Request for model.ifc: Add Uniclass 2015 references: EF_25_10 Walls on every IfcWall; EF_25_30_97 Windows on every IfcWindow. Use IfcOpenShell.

First a look at what the model holds.

```python
import ifcopenshell

model = ifcopenshell.open("model.ifc")
print(model.schema)
print("classifications:", [c.Name for c in model.by_type("IfcClassification")])
for ifc_class in ("IfcDoor", "IfcRoof", "IfcStair", "IfcWall", "IfcWindow"):
    print(ifc_class, len(model.by_type(ifc_class)))
```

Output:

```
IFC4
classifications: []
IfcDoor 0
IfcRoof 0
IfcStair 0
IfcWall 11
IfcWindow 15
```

```python
import ifcopenshell
import ifcopenshell.api.classification

model = ifcopenshell.open("model.ifc")

system = ifcopenshell.api.classification.add_classification(model, classification="Uniclass 2015")

codes = {
    "IfcWall": ("EF_25_10", "Walls"),
    "IfcWindow": ("EF_25_30_97", "Windows"),
}
for ifc_class, (code, name) in codes.items():
    products = model.by_type(ifc_class)
    ifcopenshell.api.classification.add_reference(
        model, products=products, classification=system, identification=code, name=name
    )
    print(code, len(products))

model.write("model_rev.ifc")
```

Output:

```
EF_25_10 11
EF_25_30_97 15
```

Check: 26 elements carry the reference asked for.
